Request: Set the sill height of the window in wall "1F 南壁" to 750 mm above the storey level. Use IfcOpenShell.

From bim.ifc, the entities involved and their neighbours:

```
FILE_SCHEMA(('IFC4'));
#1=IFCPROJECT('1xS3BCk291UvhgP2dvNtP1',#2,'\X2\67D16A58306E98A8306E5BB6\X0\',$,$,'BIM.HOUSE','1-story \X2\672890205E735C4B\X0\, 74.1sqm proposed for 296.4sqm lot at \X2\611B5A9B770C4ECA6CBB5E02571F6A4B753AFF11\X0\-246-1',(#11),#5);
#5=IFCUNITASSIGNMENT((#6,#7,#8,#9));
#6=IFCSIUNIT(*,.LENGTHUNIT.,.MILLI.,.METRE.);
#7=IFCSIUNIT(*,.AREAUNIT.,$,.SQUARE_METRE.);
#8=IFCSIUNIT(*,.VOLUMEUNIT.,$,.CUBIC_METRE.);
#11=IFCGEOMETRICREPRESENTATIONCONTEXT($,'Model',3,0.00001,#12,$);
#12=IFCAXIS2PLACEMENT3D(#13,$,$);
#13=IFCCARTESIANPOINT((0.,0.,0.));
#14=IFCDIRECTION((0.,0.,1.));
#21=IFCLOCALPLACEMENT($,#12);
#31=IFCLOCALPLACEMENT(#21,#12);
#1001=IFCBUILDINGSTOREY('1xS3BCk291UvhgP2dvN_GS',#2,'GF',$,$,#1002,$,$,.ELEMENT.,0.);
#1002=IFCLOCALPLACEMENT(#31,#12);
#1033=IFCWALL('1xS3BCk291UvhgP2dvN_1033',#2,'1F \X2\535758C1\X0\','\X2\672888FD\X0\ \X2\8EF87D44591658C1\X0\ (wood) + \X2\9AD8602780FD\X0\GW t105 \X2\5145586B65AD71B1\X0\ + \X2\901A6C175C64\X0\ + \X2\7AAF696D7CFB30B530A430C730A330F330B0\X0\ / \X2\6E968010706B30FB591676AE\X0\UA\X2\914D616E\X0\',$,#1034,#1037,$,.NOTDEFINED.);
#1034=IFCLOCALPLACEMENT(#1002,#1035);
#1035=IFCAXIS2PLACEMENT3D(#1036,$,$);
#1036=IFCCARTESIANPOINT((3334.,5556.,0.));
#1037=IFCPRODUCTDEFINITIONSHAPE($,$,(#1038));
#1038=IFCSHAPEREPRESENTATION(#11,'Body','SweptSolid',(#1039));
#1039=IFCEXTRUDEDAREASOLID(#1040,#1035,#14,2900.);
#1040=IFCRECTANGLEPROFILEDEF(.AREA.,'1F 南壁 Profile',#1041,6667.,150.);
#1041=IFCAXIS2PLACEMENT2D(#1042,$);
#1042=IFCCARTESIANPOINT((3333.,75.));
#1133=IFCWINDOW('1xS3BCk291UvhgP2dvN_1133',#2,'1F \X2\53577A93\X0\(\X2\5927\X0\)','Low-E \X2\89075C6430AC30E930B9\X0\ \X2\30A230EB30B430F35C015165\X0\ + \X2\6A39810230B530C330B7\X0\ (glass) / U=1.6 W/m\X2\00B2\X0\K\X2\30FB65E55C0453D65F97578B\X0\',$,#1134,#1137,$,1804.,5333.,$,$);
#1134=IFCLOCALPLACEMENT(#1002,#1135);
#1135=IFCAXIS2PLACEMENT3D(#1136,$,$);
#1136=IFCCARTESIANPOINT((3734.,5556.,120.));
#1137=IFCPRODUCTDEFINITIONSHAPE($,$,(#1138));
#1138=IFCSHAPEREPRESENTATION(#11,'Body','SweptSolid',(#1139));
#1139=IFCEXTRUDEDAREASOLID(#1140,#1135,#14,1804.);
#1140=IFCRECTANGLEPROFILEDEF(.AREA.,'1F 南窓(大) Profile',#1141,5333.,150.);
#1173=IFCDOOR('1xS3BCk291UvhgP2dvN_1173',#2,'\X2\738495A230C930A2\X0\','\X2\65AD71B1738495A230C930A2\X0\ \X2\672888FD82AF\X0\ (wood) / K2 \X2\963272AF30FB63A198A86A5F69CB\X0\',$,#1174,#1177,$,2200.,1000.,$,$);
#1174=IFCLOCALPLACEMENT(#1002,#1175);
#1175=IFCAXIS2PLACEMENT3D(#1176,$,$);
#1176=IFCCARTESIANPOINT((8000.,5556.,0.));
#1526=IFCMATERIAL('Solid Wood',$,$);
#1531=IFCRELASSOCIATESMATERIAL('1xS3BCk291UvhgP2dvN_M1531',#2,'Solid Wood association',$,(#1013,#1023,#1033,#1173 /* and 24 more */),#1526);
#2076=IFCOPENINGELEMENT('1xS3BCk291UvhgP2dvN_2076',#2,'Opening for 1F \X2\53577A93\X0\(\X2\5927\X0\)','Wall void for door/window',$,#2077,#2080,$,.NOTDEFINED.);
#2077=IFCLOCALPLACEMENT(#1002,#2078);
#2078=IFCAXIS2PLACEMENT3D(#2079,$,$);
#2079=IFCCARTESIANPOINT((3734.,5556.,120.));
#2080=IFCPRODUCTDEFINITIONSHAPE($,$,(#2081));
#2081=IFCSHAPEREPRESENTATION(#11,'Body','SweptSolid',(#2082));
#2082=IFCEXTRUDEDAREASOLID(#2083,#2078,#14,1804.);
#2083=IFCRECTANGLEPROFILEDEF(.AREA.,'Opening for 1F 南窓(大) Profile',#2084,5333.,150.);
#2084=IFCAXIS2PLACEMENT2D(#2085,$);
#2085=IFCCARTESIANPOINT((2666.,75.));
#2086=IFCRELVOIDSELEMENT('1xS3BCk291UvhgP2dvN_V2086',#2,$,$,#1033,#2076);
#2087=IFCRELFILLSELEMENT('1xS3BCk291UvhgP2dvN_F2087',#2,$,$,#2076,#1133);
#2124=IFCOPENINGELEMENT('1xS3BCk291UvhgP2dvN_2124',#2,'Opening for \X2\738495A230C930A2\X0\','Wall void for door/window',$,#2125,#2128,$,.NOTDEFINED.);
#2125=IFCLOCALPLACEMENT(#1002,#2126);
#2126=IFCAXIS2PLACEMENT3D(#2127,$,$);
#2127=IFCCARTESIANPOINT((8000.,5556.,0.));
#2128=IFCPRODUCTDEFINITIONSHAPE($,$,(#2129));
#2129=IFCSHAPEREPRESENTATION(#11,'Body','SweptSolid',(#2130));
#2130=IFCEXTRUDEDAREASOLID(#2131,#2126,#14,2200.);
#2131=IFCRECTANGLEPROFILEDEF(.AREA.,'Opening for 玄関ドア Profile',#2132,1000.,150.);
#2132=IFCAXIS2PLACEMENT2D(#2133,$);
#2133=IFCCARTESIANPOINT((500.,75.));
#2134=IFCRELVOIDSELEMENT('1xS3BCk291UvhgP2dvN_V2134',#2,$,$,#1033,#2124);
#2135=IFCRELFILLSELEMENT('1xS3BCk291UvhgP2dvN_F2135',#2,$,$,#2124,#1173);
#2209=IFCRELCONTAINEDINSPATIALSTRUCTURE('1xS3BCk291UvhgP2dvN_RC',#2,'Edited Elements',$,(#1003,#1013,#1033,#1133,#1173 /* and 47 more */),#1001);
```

```python
import numpy as np
import ifcopenshell
import ifcopenshell.api.geometry
import ifcopenshell.geom
import ifcopenshell.util.element
import ifcopenshell.util.placement
import ifcopenshell.util.shape
import ifcopenshell.util.unit

model = ifcopenshell.open("bim.ifc")
unit_scale = ifcopenshell.util.unit.calculate_unit_scale(model)

window = model.by_guid("1xS3BCk291UvhgP2dvN_1133")
opening = window.FillsVoids[0].RelatingOpeningElement
storey = ifcopenshell.util.element.get_container(window, ifc_class="IfcBuildingStorey")
level = ifcopenshell.util.placement.get_local_placement(storey.ObjectPlacement)[2, 3]

# The opening's origin need not be at the sill, so measure its lowest point.
shape = ifcopenshell.geom.create_shape(ifcopenshell.geom.settings(), opening)
bottom = ifcopenshell.util.shape.get_shape_bottom_elevation(shape, shape.geometry) / unit_scale
dz = level + 0.75 / unit_scale - bottom

shift = np.array([0.0, 0.0, dz])
# The window is not placed relative to its opening, so move both.
for product in (opening, window):
    matrix = ifcopenshell.util.placement.get_local_placement(product.ObjectPlacement)
    matrix[:3, 3] += shift
    ifcopenshell.api.geometry.edit_object_placement(model, product=product, matrix=matrix, is_si=False)

print(f"moved by {dz * unit_scale:+.3f} m")

model.write("bim_edited.ifc")
```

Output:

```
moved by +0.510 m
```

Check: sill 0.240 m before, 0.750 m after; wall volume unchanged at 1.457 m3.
